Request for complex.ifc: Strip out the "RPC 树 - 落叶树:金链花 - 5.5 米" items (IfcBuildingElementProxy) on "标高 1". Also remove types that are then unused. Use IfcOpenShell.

First a look at what the model holds.

```python
import ifcopenshell
import ifcopenshell.util.element

model = ifcopenshell.open("complex.ifc")
print(model.schema)
storey = next(s for s in model.by_type("IfcBuildingStorey") if s.Name == "标高 1")
proxies = [e for e in ifcopenshell.util.element.get_decomposition(storey) if e.is_a("IfcBuildingElementProxy")]
seen = {}
for e in proxies:
    element_type = ifcopenshell.util.element.get_type(e)
    name = element_type.Name if element_type not in (None, e) else None
    seen[name] = seen.get(name, 0) + 1
for name, count in sorted(seen.items(), key=str):
    print(count, "x", name)
```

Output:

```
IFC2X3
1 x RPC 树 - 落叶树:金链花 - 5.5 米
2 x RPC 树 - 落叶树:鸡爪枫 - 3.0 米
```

```python
import ifcopenshell
import ifcopenshell.api.root
import ifcopenshell.util.element

model = ifcopenshell.open("complex.ifc")

storey = next(s for s in model.by_type("IfcBuildingStorey") if s.Name == "标高 1")
proxies = [e for e in ifcopenshell.util.element.get_decomposition(storey) if e.is_a("IfcBuildingElementProxy")]
targets = [e for e in proxies if (t := ifcopenshell.util.element.get_type(e)) not in (None, e) and t.Name == "RPC 树 - 落叶树:金链花 - 5.5 米"]
types = {ifcopenshell.util.element.get_type(e) for e in targets} - {None, *targets}

for e in targets:
    ifcopenshell.api.root.remove_product(model, product=e)
print(len(targets), "removed")

unused = [t for t in types if not ifcopenshell.util.element.get_types(t)]
for t in unused:
    ifcopenshell.api.root.remove_product(model, product=t)
print(len(unused), "unused types removed")

model.write("complex_v2.ifc")
```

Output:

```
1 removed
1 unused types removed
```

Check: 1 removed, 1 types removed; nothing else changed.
